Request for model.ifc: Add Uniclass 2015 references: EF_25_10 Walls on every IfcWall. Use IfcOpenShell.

First a look at what the model holds.

```python
import ifcopenshell

model = ifcopenshell.open("model.ifc")
print(model.schema)
print("classifications:", [c.Name for c in model.by_type("IfcClassification")])
for ifc_class in ("IfcDoor", "IfcRoof", "IfcStair", "IfcWall", "IfcWindow"):
    print(ifc_class, len(model.by_type(ifc_class)))
```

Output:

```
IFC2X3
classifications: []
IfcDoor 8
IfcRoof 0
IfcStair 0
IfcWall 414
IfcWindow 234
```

```python
import ifcopenshell
import ifcopenshell.api.classification

model = ifcopenshell.open("model.ifc")

# IFC2X3 requires Source and Edition and has no link from the project to the system.
system = model.create_entity("IfcClassification", Source="NBS", Edition="2015", Name="Uniclass 2015")

codes = {
    "IfcWall": ("EF_25_10", "Walls"),
}
for ifc_class, (code, name) in codes.items():
    products = model.by_type(ifc_class)
    ifcopenshell.api.classification.add_reference(
        model, products=products, classification=system, identification=code, name=name
    )
    print(code, len(products))

model.write("model_updated.ifc")
```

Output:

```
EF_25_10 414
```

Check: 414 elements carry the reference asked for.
